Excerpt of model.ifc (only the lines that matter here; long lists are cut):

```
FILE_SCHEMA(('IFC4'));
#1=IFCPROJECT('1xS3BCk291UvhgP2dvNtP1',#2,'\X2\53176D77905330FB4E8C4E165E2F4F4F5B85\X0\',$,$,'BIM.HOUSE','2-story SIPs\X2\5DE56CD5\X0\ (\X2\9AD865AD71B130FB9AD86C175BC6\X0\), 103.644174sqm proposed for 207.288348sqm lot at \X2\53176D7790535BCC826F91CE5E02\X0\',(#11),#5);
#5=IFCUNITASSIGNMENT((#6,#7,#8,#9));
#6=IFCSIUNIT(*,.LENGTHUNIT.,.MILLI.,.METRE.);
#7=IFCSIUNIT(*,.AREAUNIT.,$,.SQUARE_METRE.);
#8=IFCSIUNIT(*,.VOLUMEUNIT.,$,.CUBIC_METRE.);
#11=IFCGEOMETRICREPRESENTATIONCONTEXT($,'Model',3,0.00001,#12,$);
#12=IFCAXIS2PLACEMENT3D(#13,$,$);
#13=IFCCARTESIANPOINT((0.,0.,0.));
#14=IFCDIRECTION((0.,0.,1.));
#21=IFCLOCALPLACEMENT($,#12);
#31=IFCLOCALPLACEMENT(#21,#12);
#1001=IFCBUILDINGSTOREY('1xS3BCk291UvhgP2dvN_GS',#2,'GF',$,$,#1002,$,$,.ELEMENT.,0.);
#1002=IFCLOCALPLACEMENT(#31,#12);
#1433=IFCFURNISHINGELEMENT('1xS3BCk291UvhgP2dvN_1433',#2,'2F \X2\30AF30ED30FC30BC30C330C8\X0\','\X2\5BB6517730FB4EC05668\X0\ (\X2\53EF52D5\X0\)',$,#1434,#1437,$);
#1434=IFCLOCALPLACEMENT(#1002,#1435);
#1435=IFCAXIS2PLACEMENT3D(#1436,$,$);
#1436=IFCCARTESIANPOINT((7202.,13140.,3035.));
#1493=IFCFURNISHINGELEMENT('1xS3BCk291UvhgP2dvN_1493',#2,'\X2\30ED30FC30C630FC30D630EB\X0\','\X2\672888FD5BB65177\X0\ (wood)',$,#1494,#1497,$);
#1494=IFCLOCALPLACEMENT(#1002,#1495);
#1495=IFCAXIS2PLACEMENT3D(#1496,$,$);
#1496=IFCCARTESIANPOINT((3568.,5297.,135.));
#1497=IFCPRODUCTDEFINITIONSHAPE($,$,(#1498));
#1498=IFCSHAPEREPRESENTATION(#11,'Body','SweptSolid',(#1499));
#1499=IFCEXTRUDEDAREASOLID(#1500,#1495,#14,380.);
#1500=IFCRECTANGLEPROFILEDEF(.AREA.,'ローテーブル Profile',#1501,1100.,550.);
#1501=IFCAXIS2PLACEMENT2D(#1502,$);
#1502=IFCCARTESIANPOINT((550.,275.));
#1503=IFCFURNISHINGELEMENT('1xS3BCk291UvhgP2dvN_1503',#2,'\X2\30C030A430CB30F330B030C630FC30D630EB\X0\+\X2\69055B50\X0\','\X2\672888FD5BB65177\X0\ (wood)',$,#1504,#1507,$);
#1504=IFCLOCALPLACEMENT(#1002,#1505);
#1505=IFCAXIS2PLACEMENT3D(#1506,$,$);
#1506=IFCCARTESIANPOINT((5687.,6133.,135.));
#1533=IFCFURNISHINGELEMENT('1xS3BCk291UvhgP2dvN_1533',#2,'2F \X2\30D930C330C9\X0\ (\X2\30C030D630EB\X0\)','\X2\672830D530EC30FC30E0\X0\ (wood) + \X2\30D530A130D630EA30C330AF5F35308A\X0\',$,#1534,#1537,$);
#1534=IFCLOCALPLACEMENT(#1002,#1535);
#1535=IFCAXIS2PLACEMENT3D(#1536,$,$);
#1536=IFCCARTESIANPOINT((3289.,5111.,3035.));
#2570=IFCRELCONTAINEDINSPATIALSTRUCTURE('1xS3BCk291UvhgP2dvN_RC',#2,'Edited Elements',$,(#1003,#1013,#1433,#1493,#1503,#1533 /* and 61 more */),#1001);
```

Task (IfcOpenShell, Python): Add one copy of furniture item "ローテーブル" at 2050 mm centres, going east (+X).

```python
import numpy as np
import ifcopenshell
import ifcopenshell.api.geometry
import ifcopenshell.api.root
import ifcopenshell.util.element
import ifcopenshell.util.placement

model = ifcopenshell.open("model.ifc")


def reuse_history(source, copy):
    """copy_class also copies each property set's owner history, people and application; keep the originals."""
    for rel in copy.IsDefinedBy:
        if rel.is_a("IfcRelDefinesByProperties") and (history := rel.RelatingPropertyDefinition.OwnerHistory):
            rel.RelatingPropertyDefinition.OwnerHistory = source.OwnerHistory
            ifcopenshell.util.element.remove_deep2(model, history)


source = model.by_id(1493)
base = ifcopenshell.util.placement.get_local_placement(source.ObjectPlacement)
step = np.array([1.0, 0.0, 0.0]) * 2050.0

for i in range(1, 2):
    copy = ifcopenshell.api.root.copy_class(model, product=source)
    copy.Representation = ifcopenshell.util.element.copy_deep(
        model, source.Representation, exclude=["IfcGeometricRepresentationContext", "IfcRepresentationMap"]
    )
    reuse_history(source, copy)
    matrix = base.copy()
    matrix[:3, 3] += i * step
    print("added at", matrix[:3, 3].round(3) + 0.0)
    ifcopenshell.api.geometry.edit_object_placement(model, product=copy, matrix=matrix, is_si=False)

model.write("model_rev.ifc")
```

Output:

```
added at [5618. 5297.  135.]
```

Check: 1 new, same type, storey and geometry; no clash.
